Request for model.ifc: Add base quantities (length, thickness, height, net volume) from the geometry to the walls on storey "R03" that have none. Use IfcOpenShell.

First a look at what the model holds.

```python
import ifcopenshell
import ifcopenshell.util.element
import ifcopenshell.util.unit

model = ifcopenshell.open("model.ifc")
print(model.schema)
for unit_type in ("LENGTHUNIT", "AREAUNIT", "VOLUMEUNIT"):
    print(unit_type, ifcopenshell.util.unit.calculate_unit_scale(model, unit_type))
storey = next(s for s in model.by_type("IfcBuildingStorey") if s.Name == "R03")
walls = [e for e in ifcopenshell.util.element.get_decomposition(storey) if e.is_a("IfcWall")]
for e in sorted(walls, key=lambda e: e.id()):
    print(e.id(), e.is_a(), e.Name, list(ifcopenshell.util.element.get_psets(e, qtos_only=True)), sep=" | ")
```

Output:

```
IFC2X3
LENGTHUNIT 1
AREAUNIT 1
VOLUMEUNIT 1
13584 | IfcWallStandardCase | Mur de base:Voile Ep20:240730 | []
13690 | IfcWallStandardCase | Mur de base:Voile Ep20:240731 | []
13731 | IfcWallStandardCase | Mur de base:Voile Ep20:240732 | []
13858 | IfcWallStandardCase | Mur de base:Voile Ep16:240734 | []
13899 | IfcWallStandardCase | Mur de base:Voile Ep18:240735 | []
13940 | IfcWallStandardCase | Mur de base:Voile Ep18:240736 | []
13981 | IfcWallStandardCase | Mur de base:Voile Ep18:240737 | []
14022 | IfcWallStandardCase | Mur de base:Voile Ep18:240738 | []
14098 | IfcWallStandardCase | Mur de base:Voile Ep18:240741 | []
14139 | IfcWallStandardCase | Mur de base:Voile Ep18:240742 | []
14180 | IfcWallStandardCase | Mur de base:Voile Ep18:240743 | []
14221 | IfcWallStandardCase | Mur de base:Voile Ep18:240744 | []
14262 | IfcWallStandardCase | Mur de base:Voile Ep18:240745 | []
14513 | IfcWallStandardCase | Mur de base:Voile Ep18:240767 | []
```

```python
import ifcopenshell
import ifcopenshell.api.pset
import ifcopenshell.geom
import ifcopenshell.util.element
import ifcopenshell.util.shape
import ifcopenshell.util.unit

model = ifcopenshell.open("model.ifc")
unit_scale = ifcopenshell.util.unit.calculate_unit_scale(model)
volume_scale = ifcopenshell.util.unit.calculate_unit_scale(model, "VOLUMEUNIT")
settings = ifcopenshell.geom.settings()

storey = next(s for s in model.by_type("IfcBuildingStorey") if s.Name == "R03")
walls = [e for e in ifcopenshell.util.element.get_decomposition(storey) if e.is_a("IfcWall")]

for e in sorted(walls, key=lambda e: e.id()):
    if ifcopenshell.util.element.get_psets(e, qtos_only=True, should_inherit=False):
        continue
    # Geometry comes back in metres, in the element's own axes.
    shape = ifcopenshell.geom.create_shape(settings, e)
    values = {
        "Length": ifcopenshell.util.shape.get_x(shape.geometry) / unit_scale,
        "Width": ifcopenshell.util.shape.get_y(shape.geometry) / unit_scale,
        "Height": ifcopenshell.util.shape.get_z(shape.geometry) / unit_scale,
        "NetVolume": ifcopenshell.util.shape.get_volume(shape.geometry) / volume_scale,
    }
    qto = ifcopenshell.api.pset.add_qto(model, product=e, name="BaseQuantities")
    ifcopenshell.api.pset.edit_qto(model, qto=qto, properties=values)
    print(e.id(), {k: round(v, 3) for k, v in values.items()})

model.write("model_v2.ifc")
```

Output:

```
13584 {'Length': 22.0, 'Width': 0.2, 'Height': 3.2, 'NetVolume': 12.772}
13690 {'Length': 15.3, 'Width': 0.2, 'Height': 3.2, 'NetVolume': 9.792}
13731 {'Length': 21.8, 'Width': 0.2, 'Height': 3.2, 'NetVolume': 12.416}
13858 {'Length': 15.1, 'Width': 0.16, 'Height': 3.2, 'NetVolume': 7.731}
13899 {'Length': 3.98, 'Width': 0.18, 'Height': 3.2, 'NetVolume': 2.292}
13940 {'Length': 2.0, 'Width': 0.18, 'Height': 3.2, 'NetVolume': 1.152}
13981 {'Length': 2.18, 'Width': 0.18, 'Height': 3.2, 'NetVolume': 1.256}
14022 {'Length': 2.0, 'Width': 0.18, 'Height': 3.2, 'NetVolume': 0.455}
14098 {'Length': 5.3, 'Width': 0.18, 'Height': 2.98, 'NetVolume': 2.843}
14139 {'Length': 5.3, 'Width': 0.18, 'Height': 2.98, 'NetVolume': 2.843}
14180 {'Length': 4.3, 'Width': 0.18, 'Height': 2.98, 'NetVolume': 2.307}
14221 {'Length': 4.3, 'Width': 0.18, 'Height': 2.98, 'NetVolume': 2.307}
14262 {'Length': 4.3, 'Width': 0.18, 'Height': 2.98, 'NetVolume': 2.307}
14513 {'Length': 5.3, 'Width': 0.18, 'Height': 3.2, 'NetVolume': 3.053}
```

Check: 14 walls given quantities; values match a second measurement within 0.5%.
